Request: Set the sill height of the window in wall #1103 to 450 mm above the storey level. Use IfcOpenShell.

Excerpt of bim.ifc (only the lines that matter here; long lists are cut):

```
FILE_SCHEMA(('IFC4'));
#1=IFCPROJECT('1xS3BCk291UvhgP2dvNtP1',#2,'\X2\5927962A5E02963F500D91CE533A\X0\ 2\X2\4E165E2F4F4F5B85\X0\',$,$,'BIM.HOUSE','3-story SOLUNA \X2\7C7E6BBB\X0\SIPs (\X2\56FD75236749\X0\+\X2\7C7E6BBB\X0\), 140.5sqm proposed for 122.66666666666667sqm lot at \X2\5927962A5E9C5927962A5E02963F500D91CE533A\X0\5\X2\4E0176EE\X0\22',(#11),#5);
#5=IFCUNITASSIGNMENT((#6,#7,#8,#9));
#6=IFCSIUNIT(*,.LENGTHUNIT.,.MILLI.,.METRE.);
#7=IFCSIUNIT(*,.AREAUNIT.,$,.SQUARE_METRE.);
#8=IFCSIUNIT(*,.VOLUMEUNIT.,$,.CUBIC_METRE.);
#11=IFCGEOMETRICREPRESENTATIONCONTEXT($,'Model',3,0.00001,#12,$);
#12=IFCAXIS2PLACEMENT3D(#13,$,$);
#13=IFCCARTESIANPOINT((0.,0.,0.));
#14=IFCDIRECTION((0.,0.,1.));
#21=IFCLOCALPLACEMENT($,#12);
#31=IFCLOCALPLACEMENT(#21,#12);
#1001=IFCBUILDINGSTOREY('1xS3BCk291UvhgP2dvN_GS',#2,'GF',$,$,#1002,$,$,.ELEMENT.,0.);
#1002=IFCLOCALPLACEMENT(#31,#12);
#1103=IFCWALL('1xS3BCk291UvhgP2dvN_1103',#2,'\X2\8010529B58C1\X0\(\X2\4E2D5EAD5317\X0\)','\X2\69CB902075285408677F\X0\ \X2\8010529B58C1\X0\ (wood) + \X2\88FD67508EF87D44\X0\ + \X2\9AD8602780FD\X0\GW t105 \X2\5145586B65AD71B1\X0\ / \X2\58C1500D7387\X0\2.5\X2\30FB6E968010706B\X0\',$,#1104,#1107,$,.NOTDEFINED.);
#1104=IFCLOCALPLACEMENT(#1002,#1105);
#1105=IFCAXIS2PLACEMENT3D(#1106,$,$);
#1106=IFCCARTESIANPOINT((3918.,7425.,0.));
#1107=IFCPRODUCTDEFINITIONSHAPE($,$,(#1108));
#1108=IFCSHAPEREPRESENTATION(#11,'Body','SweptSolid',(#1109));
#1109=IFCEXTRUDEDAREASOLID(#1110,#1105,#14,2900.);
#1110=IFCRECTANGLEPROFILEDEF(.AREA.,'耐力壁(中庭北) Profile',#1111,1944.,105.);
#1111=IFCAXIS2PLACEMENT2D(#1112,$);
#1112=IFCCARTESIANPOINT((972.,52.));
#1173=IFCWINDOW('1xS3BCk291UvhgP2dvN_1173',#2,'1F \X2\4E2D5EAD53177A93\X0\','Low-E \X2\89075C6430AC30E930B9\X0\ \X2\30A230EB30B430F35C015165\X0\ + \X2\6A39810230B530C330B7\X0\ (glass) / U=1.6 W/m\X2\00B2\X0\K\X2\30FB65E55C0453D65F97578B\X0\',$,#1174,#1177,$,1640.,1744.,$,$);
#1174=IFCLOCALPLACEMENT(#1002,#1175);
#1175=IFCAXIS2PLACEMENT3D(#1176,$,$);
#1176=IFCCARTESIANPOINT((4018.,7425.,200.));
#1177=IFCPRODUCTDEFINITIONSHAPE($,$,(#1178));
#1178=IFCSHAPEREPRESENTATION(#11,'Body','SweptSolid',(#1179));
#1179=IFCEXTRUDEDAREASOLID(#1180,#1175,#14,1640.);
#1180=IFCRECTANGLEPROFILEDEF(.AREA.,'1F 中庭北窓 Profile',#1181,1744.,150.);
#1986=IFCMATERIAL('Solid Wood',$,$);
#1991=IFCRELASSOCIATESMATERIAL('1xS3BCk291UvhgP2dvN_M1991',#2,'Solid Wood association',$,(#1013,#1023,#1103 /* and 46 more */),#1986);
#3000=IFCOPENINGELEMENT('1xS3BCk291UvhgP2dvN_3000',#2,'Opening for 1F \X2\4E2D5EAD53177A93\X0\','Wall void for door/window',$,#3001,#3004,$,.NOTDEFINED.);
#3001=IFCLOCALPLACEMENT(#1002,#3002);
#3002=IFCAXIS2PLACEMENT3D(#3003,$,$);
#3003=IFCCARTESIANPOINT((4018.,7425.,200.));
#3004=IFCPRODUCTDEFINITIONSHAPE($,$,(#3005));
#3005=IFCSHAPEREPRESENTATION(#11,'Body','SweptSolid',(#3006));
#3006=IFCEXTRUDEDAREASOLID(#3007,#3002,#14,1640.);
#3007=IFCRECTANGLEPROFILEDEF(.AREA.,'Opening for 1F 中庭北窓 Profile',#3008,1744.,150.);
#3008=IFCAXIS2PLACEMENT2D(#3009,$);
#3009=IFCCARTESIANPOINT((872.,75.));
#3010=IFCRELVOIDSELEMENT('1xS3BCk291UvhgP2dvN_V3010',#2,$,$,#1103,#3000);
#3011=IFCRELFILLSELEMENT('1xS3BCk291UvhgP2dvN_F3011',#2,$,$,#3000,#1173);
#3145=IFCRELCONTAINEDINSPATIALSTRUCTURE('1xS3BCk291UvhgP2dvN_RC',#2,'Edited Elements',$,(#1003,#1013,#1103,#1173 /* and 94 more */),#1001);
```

```python
import numpy as np
import ifcopenshell
import ifcopenshell.api.geometry
import ifcopenshell.geom
import ifcopenshell.util.element
import ifcopenshell.util.placement
import ifcopenshell.util.shape
import ifcopenshell.util.unit

model = ifcopenshell.open("bim.ifc")
unit_scale = ifcopenshell.util.unit.calculate_unit_scale(model)

window = model.by_guid("1xS3BCk291UvhgP2dvN_1173")
opening = window.FillsVoids[0].RelatingOpeningElement
storey = ifcopenshell.util.element.get_container(window, ifc_class="IfcBuildingStorey")
level = ifcopenshell.util.placement.get_local_placement(storey.ObjectPlacement)[2, 3]

# The opening's origin need not be at the sill, so measure its lowest point.
shape = ifcopenshell.geom.create_shape(ifcopenshell.geom.settings(), opening)
bottom = ifcopenshell.util.shape.get_shape_bottom_elevation(shape, shape.geometry) / unit_scale
dz = level + 450.0 - bottom

shift = np.array([0.0, 0.0, dz])
# The window is not placed relative to its opening, so move both.
for product in (opening, window):
    matrix = ifcopenshell.util.placement.get_local_placement(product.ObjectPlacement)
    matrix[:3, 3] += shift
    ifcopenshell.api.geometry.edit_object_placement(model, product=product, matrix=matrix, is_si=False)

print(f"moved by {dz * unit_scale:+.3f} m")

model.write("bim_edited.ifc")
```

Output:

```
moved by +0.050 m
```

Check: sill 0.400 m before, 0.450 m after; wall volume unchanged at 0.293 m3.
